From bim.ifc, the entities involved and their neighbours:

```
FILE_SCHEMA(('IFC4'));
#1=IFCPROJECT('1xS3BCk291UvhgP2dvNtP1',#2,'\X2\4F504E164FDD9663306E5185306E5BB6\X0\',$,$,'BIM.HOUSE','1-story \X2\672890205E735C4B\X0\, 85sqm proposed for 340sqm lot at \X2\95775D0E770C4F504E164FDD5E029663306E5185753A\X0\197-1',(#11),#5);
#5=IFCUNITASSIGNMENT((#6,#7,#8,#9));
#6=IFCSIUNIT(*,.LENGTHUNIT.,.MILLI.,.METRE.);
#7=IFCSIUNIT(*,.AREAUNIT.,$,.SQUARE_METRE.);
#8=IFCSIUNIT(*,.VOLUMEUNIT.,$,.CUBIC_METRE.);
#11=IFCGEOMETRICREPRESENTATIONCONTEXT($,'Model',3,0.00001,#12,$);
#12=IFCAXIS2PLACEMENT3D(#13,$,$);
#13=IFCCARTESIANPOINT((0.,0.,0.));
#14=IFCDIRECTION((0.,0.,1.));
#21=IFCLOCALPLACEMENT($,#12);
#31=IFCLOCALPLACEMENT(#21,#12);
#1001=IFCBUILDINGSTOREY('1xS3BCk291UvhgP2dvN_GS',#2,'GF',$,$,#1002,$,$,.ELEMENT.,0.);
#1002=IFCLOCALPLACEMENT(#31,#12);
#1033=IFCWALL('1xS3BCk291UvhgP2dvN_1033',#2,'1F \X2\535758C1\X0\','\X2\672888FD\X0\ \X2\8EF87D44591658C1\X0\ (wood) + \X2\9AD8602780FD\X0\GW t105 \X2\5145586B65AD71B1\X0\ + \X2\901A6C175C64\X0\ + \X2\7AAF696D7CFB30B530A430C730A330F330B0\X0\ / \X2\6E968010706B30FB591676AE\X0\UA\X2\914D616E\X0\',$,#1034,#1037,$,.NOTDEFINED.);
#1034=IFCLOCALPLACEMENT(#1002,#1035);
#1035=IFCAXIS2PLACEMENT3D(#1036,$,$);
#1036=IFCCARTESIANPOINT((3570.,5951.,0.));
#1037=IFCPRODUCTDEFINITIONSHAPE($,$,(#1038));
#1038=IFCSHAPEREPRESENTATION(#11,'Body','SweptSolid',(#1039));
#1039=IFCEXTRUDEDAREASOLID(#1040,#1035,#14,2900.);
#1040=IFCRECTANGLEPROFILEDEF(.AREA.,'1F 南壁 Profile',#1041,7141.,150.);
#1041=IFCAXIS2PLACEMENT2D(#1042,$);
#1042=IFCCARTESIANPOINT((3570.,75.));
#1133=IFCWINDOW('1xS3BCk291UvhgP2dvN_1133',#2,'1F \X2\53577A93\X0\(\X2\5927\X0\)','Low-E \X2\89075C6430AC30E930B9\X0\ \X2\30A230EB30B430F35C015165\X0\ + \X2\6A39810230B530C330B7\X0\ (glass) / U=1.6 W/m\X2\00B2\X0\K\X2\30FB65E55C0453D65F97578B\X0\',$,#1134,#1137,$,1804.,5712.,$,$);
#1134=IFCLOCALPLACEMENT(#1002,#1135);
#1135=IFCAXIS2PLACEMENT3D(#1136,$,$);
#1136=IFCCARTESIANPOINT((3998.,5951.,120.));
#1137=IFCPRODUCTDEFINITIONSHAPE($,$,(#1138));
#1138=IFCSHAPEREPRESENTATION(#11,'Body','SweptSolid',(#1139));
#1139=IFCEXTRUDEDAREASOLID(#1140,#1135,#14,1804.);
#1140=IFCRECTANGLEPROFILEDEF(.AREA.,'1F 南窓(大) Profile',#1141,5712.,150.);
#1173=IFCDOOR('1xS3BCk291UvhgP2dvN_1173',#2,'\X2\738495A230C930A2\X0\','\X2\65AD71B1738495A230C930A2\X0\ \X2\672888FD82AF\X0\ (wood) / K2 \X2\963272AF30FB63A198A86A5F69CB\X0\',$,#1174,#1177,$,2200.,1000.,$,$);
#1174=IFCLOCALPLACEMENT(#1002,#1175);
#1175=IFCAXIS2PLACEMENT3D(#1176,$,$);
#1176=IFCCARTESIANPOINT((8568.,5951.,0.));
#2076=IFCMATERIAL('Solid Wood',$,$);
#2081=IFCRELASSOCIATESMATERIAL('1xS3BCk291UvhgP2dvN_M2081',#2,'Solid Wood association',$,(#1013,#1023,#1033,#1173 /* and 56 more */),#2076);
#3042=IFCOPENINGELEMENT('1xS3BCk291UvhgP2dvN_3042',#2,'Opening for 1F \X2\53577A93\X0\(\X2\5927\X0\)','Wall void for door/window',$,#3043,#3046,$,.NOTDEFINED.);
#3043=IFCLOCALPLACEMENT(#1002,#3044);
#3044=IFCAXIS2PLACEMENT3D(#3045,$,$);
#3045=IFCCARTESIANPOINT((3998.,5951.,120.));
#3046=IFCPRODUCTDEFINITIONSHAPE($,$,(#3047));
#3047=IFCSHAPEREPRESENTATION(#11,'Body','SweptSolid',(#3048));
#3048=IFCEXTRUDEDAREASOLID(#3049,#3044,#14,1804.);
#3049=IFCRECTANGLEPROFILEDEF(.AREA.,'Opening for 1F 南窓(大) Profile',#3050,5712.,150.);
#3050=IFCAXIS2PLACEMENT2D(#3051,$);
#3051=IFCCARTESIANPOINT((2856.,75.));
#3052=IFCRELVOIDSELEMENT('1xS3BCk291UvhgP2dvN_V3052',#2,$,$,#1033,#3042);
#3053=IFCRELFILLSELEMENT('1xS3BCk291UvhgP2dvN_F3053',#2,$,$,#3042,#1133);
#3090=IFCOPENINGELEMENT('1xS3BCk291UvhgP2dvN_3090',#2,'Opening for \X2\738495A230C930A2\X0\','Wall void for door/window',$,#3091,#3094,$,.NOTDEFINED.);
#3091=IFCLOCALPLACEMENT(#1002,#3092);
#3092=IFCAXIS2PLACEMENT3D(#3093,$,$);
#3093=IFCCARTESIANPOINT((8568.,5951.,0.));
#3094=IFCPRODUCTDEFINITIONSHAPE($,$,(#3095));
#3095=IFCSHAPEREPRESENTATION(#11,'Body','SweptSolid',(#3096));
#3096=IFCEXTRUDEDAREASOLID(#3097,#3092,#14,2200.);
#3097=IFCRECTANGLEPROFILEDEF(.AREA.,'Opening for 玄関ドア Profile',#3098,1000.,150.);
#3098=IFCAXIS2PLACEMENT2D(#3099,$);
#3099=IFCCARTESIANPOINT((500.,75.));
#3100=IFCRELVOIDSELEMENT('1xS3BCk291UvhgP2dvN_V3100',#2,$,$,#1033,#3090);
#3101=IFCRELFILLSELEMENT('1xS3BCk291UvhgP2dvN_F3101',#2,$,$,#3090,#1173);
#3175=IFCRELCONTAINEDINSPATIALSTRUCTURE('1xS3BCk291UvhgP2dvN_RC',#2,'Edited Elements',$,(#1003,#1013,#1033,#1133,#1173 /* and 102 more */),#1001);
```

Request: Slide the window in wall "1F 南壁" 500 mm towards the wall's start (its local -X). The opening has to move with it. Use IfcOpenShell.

```python
import ifcopenshell
import ifcopenshell.api.geometry
import ifcopenshell.util.placement

model = ifcopenshell.open("bim.ifc")

window = model.by_guid("1xS3BCk291UvhgP2dvN_1133")
opening = window.FillsVoids[0].RelatingOpeningElement
wall = opening.VoidsElements[0].RelatingBuildingElement

wall_matrix = ifcopenshell.util.placement.get_local_placement(wall.ObjectPlacement)
shift = wall_matrix[:3, 0] * -500.0
before = ifcopenshell.util.placement.get_local_placement(window.ObjectPlacement)[:3, 3].copy()

# The window is not placed relative to its opening, so move both.
for product in (opening, window):
    matrix = ifcopenshell.util.placement.get_local_placement(product.ObjectPlacement)
    matrix[:3, 3] += shift
    ifcopenshell.api.geometry.edit_object_placement(model, product=product, matrix=matrix, is_si=False)

after = ifcopenshell.util.placement.get_local_placement(window.ObjectPlacement)[:3, 3]
print("window moved by", (after - before).round(3) + 0.0)

model.write("bim_updated.ifc")
```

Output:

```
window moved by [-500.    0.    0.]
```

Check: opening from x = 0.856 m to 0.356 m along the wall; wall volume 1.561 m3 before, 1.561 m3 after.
